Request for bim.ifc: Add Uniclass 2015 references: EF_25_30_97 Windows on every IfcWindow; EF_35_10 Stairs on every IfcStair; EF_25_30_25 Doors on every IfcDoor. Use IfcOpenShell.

First a look at what the model holds.

```python
import ifcopenshell

model = ifcopenshell.open("bim.ifc")
print(model.schema)
print("classifications:", [c.Name for c in model.by_type("IfcClassification")])
for ifc_class in ("IfcDoor", "IfcRoof", "IfcStair", "IfcWall", "IfcWindow"):
    print(ifc_class, len(model.by_type(ifc_class)))
```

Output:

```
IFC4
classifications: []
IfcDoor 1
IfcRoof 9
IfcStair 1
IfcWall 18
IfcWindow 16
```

```python
import ifcopenshell
import ifcopenshell.api.classification

model = ifcopenshell.open("bim.ifc")

system = ifcopenshell.api.classification.add_classification(model, classification="Uniclass 2015")

codes = {
    "IfcWindow": ("EF_25_30_97", "Windows"),
    "IfcStair": ("EF_35_10", "Stairs"),
    "IfcDoor": ("EF_25_30_25", "Doors"),
}
for ifc_class, (code, name) in codes.items():
    products = model.by_type(ifc_class)
    ifcopenshell.api.classification.add_reference(
        model, products=products, classification=system, identification=code, name=name
    )
    print(code, len(products))

model.write("bim_rev.ifc")
```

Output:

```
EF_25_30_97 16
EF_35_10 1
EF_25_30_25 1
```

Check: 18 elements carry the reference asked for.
